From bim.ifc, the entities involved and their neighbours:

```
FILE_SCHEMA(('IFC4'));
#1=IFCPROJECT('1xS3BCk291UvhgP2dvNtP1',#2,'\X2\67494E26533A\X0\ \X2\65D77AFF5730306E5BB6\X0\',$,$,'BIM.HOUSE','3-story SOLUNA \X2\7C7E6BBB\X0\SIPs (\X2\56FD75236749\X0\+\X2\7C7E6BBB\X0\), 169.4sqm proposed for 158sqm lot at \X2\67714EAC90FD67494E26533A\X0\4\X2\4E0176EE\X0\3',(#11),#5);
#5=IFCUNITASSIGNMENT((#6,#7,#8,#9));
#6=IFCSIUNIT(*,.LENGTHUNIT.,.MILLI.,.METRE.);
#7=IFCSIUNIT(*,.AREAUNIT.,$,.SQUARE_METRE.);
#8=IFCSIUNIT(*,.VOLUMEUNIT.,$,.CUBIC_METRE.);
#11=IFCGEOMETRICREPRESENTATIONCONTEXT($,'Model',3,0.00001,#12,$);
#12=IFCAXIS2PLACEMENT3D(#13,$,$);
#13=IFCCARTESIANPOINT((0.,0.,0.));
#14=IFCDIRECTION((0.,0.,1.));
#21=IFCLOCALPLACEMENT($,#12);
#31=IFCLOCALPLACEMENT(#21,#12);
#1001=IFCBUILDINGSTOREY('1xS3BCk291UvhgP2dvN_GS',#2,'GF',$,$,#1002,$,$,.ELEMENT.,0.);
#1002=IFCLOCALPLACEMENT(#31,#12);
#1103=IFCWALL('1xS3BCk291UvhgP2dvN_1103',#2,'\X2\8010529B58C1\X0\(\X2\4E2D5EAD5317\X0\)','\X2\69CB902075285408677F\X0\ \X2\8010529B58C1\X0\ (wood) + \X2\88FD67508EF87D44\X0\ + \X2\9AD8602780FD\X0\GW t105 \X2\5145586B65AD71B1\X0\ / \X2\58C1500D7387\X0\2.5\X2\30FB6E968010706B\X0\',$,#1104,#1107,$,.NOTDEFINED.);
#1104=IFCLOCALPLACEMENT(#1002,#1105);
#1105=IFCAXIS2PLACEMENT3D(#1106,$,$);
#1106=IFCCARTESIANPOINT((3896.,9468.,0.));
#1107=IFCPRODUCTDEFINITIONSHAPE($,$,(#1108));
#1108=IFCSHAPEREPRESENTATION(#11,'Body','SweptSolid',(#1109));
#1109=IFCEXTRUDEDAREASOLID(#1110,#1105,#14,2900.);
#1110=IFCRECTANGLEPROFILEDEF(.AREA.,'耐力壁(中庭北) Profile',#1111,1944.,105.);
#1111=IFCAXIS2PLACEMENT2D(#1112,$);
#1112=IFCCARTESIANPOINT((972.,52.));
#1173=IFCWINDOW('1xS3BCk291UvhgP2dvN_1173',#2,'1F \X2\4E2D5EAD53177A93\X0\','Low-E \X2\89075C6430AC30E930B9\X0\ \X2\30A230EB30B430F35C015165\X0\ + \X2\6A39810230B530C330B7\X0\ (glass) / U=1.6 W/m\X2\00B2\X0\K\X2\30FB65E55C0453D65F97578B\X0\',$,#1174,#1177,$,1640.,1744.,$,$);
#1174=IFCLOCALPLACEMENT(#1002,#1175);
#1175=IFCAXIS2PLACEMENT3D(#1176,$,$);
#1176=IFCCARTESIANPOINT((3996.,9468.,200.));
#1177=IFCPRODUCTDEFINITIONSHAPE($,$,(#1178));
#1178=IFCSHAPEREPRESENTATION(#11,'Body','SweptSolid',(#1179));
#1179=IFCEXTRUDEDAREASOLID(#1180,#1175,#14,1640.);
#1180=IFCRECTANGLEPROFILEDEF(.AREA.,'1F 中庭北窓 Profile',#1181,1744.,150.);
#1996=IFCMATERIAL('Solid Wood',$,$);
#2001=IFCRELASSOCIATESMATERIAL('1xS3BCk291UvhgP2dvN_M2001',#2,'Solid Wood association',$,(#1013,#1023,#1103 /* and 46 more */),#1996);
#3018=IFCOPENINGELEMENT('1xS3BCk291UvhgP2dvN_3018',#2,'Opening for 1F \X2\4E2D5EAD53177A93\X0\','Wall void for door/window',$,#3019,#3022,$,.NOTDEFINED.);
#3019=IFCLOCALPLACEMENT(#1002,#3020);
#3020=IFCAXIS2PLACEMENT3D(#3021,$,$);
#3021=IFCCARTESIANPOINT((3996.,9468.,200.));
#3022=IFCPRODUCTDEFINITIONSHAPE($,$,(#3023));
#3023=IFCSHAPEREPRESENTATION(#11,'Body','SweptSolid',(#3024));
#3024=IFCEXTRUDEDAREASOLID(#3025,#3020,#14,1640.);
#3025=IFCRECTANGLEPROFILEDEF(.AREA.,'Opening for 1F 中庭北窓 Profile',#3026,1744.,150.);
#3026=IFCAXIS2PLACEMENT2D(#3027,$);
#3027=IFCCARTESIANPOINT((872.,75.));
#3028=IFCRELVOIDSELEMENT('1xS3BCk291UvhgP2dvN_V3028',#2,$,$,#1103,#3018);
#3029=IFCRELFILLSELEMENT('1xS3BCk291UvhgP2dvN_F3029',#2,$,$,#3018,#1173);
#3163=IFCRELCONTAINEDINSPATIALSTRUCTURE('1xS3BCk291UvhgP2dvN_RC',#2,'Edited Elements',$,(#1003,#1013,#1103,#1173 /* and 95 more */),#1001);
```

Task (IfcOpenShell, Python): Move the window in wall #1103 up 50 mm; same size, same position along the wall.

```python
import numpy as np
import ifcopenshell
import ifcopenshell.api.geometry
import ifcopenshell.util.placement
import ifcopenshell.util.unit

model = ifcopenshell.open("bim.ifc")
unit_scale = ifcopenshell.util.unit.calculate_unit_scale(model)

window = model.by_guid("1xS3BCk291UvhgP2dvN_1173")
opening = window.FillsVoids[0].RelatingOpeningElement
dz = 0.05 / unit_scale

shift = np.array([0.0, 0.0, dz])
# The window is not placed relative to its opening, so move both.
for product in (opening, window):
    matrix = ifcopenshell.util.placement.get_local_placement(product.ObjectPlacement)
    matrix[:3, 3] += shift
    ifcopenshell.api.geometry.edit_object_placement(model, product=product, matrix=matrix, is_si=False)

print(f"moved by {dz * unit_scale:+.3f} m")

model.write("bim_updated.ifc")
```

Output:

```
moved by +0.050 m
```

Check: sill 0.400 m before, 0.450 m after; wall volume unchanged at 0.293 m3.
